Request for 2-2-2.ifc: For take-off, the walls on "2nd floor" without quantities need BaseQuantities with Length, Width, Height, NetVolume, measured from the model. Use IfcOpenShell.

First a look at what the model holds.

```python
import ifcopenshell
import ifcopenshell.util.element
import ifcopenshell.util.unit

model = ifcopenshell.open("2-2-2.ifc")
print(model.schema)
for unit_type in ("LENGTHUNIT", "AREAUNIT", "VOLUMEUNIT"):
    print(unit_type, ifcopenshell.util.unit.calculate_unit_scale(model, unit_type))
storey = next(s for s in model.by_type("IfcBuildingStorey") if s.Name == "2nd floor")
walls = [e for e in ifcopenshell.util.element.get_decomposition(storey) if e.is_a("IfcWall")]
for e in sorted(walls, key=lambda e: e.id()):
    print(e.id(), e.is_a(), e.Name, list(ifcopenshell.util.element.get_psets(e, qtos_only=True)), sep=" | ")
```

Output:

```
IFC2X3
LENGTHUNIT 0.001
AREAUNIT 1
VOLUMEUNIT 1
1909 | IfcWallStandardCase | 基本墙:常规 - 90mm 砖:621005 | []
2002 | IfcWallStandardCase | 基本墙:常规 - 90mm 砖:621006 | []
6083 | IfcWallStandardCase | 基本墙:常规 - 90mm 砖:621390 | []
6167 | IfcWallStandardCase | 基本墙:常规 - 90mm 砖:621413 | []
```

```python
import ifcopenshell
import ifcopenshell.api.pset
import ifcopenshell.geom
import ifcopenshell.util.element
import ifcopenshell.util.shape
import ifcopenshell.util.unit

model = ifcopenshell.open("2-2-2.ifc")
unit_scale = ifcopenshell.util.unit.calculate_unit_scale(model)
volume_scale = ifcopenshell.util.unit.calculate_unit_scale(model, "VOLUMEUNIT")
settings = ifcopenshell.geom.settings()

storey = next(s for s in model.by_type("IfcBuildingStorey") if s.Name == "2nd floor")
walls = [e for e in ifcopenshell.util.element.get_decomposition(storey) if e.is_a("IfcWall")]

for e in sorted(walls, key=lambda e: e.id()):
    if ifcopenshell.util.element.get_psets(e, qtos_only=True, should_inherit=False):
        continue
    # Geometry comes back in metres, in the element's own axes.
    shape = ifcopenshell.geom.create_shape(settings, e)
    values = {
        "Length": ifcopenshell.util.shape.get_x(shape.geometry) / unit_scale,
        "Width": ifcopenshell.util.shape.get_y(shape.geometry) / unit_scale,
        "Height": ifcopenshell.util.shape.get_z(shape.geometry) / unit_scale,
        "NetVolume": ifcopenshell.util.shape.get_volume(shape.geometry) / volume_scale,
    }
    qto = ifcopenshell.api.pset.add_qto(model, product=e, name="BaseQuantities")
    ifcopenshell.api.pset.edit_qto(model, qto=qto, properties=values)
    print(e.id(), {k: round(v, 3) for k, v in values.items()})

model.write("2-2-2-out.ifc")
```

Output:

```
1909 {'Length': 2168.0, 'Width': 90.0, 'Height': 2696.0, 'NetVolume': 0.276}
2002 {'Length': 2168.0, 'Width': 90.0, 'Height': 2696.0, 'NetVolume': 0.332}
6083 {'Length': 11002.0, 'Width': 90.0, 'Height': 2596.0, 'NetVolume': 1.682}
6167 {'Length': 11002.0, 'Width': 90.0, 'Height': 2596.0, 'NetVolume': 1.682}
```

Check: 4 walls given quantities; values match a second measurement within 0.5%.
